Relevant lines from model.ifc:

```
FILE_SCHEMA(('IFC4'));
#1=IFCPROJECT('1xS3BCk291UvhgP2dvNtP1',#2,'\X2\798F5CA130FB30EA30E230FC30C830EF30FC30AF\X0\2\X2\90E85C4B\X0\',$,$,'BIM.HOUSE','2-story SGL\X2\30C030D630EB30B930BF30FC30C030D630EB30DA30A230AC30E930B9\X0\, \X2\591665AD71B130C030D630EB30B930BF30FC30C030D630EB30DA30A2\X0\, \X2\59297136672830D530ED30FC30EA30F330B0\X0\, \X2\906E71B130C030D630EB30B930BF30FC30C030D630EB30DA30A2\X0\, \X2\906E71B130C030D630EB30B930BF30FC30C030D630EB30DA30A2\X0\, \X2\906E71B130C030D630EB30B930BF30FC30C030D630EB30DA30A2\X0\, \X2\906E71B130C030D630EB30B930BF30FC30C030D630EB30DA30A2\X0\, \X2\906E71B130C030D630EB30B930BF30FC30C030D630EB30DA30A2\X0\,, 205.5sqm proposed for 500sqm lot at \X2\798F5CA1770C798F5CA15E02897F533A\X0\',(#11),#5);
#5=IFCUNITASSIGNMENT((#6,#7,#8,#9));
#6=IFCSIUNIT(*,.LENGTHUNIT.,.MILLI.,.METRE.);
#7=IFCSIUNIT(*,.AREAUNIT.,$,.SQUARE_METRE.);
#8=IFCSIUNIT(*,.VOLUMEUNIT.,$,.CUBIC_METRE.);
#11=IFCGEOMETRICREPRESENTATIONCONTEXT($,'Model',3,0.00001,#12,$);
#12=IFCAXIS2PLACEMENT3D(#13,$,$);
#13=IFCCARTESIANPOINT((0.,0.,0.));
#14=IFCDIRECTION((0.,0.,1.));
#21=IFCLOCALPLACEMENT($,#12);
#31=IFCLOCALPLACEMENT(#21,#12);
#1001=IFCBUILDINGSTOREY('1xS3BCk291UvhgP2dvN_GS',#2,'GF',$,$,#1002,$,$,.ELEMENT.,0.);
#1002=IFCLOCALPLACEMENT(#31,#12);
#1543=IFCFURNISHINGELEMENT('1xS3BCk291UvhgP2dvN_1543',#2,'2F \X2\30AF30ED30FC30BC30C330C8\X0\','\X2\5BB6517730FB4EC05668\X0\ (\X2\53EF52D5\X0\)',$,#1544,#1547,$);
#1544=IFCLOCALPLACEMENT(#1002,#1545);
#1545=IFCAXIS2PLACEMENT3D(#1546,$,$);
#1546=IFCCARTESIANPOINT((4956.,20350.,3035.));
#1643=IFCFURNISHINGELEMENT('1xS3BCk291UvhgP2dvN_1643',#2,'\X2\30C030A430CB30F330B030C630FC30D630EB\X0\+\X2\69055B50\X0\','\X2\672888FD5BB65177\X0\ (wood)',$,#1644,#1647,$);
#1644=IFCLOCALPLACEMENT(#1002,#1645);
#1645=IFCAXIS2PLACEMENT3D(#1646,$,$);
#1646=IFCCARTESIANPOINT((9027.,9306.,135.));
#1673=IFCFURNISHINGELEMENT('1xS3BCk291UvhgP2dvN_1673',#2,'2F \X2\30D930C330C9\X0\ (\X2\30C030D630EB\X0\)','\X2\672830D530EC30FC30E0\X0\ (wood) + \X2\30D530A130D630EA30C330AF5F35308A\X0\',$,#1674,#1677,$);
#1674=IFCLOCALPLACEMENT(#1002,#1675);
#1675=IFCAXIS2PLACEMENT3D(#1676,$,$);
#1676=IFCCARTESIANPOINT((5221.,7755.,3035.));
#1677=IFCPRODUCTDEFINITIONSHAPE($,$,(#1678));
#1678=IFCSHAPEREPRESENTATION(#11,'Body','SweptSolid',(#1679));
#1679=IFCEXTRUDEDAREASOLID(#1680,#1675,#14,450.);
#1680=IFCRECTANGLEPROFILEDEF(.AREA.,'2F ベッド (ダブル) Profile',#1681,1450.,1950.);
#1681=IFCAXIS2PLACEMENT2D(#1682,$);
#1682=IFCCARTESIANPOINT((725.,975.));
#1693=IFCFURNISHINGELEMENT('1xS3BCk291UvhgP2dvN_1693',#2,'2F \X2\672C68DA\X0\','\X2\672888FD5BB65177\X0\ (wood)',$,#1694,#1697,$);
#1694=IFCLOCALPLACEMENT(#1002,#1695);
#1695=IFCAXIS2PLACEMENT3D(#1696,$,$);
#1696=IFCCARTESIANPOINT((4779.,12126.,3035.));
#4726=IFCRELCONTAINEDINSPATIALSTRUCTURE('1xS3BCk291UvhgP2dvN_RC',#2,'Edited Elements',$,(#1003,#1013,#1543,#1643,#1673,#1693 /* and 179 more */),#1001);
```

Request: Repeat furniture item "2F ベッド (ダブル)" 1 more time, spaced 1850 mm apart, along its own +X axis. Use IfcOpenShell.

```python
import ifcopenshell
import ifcopenshell.api.geometry
import ifcopenshell.api.root
import ifcopenshell.util.element
import ifcopenshell.util.placement
import ifcopenshell.util.unit

model = ifcopenshell.open("model.ifc")
unit_scale = ifcopenshell.util.unit.calculate_unit_scale(model)


def reuse_history(source, copy):
    """copy_class also copies each property set's owner history, people and application; keep the originals."""
    for rel in copy.IsDefinedBy:
        if rel.is_a("IfcRelDefinesByProperties") and (history := rel.RelatingPropertyDefinition.OwnerHistory):
            rel.RelatingPropertyDefinition.OwnerHistory = source.OwnerHistory
            ifcopenshell.util.element.remove_deep2(model, history)


source = model.by_id(1673)
base = ifcopenshell.util.placement.get_local_placement(source.ObjectPlacement)
step = base[:3, 0] * 1.85 / unit_scale

for i in range(1, 2):
    copy = ifcopenshell.api.root.copy_class(model, product=source)
    copy.Representation = ifcopenshell.util.element.copy_deep(
        model, source.Representation, exclude=["IfcGeometricRepresentationContext", "IfcRepresentationMap"]
    )
    reuse_history(source, copy)
    matrix = base.copy()
    matrix[:3, 3] += i * step
    print("added at", matrix[:3, 3].round(3) + 0.0)
    ifcopenshell.api.geometry.edit_object_placement(model, product=copy, matrix=matrix, is_si=False)

model.write("model_updated.ifc")
```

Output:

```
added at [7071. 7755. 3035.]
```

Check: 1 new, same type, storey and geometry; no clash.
